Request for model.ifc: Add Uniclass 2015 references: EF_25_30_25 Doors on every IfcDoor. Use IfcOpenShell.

First a look at what the model holds.

```python
import ifcopenshell

model = ifcopenshell.open("model.ifc")
print(model.schema)
print("classifications:", [c.Name for c in model.by_type("IfcClassification")])
for ifc_class in ("IfcDoor", "IfcRoof", "IfcStair", "IfcWall", "IfcWindow"):
    print(ifc_class, len(model.by_type(ifc_class)))
```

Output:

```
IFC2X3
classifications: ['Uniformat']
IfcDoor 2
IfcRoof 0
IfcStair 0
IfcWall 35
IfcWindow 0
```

```python
import ifcopenshell
import ifcopenshell.api.classification

model = ifcopenshell.open("model.ifc")

# IFC2X3 requires Source and Edition and has no link from the project to the system.
system = model.create_entity("IfcClassification", Source="NBS", Edition="2015", Name="Uniclass 2015")

codes = {
    "IfcDoor": ("EF_25_30_25", "Doors"),
}
for ifc_class, (code, name) in codes.items():
    products = model.by_type(ifc_class)
    ifcopenshell.api.classification.add_reference(
        model, products=products, classification=system, identification=code, name=name
    )
    print(code, len(products))

model.write("model_updated.ifc")
```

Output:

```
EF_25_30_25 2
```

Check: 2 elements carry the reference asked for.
